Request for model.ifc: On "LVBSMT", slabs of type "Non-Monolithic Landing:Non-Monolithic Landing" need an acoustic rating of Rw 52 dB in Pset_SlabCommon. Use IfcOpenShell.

First a look at what the model holds.

```python
import ifcopenshell
import ifcopenshell.util.element

model = ifcopenshell.open("model.ifc")
print(model.schema)
storey = next(s for s in model.by_type("IfcBuildingStorey") if s.Name == "LVBSMT")
slabs = [e for e in ifcopenshell.util.element.get_decomposition(storey) if e.is_a("IfcSlab")]
seen = {}
for e in slabs:
    element_type = ifcopenshell.util.element.get_type(e)
    key = (element_type.Name if element_type != e and element_type else None, ifcopenshell.util.element.get_pset(e, "Pset_SlabCommon", "AcousticRating"))
    seen[key] = seen.get(key, 0) + 1
for (name, value), count in sorted(seen.items(), key=str):
    print(count, "x", name, "|", value)
```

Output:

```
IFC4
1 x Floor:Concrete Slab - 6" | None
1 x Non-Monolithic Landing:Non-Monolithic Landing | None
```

```python
import ifcopenshell
import ifcopenshell.api.pset
import ifcopenshell.util.element

model = ifcopenshell.open("model.ifc")

storey = next(s for s in model.by_type("IfcBuildingStorey") if s.Name == "LVBSMT")
slabs = [e for e in ifcopenshell.util.element.get_decomposition(storey) if e.is_a("IfcSlab")]

count = 0
for e in slabs:
    element_type = ifcopenshell.util.element.get_type(e)
    if element_type in (None, e) or element_type.Name != "Non-Monolithic Landing:Non-Monolithic Landing":
        continue
    # add_pset returns the element's existing set when there is one.
    pset = ifcopenshell.api.pset.add_pset(model, product=e, name="Pset_SlabCommon")
    ifcopenshell.api.pset.edit_pset(model, pset=pset, properties={"AcousticRating": "Rw 52 dB"})
    count += 1

print(count, "slabs updated")

model.write("model_updated.ifc")
```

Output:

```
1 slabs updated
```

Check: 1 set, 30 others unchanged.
